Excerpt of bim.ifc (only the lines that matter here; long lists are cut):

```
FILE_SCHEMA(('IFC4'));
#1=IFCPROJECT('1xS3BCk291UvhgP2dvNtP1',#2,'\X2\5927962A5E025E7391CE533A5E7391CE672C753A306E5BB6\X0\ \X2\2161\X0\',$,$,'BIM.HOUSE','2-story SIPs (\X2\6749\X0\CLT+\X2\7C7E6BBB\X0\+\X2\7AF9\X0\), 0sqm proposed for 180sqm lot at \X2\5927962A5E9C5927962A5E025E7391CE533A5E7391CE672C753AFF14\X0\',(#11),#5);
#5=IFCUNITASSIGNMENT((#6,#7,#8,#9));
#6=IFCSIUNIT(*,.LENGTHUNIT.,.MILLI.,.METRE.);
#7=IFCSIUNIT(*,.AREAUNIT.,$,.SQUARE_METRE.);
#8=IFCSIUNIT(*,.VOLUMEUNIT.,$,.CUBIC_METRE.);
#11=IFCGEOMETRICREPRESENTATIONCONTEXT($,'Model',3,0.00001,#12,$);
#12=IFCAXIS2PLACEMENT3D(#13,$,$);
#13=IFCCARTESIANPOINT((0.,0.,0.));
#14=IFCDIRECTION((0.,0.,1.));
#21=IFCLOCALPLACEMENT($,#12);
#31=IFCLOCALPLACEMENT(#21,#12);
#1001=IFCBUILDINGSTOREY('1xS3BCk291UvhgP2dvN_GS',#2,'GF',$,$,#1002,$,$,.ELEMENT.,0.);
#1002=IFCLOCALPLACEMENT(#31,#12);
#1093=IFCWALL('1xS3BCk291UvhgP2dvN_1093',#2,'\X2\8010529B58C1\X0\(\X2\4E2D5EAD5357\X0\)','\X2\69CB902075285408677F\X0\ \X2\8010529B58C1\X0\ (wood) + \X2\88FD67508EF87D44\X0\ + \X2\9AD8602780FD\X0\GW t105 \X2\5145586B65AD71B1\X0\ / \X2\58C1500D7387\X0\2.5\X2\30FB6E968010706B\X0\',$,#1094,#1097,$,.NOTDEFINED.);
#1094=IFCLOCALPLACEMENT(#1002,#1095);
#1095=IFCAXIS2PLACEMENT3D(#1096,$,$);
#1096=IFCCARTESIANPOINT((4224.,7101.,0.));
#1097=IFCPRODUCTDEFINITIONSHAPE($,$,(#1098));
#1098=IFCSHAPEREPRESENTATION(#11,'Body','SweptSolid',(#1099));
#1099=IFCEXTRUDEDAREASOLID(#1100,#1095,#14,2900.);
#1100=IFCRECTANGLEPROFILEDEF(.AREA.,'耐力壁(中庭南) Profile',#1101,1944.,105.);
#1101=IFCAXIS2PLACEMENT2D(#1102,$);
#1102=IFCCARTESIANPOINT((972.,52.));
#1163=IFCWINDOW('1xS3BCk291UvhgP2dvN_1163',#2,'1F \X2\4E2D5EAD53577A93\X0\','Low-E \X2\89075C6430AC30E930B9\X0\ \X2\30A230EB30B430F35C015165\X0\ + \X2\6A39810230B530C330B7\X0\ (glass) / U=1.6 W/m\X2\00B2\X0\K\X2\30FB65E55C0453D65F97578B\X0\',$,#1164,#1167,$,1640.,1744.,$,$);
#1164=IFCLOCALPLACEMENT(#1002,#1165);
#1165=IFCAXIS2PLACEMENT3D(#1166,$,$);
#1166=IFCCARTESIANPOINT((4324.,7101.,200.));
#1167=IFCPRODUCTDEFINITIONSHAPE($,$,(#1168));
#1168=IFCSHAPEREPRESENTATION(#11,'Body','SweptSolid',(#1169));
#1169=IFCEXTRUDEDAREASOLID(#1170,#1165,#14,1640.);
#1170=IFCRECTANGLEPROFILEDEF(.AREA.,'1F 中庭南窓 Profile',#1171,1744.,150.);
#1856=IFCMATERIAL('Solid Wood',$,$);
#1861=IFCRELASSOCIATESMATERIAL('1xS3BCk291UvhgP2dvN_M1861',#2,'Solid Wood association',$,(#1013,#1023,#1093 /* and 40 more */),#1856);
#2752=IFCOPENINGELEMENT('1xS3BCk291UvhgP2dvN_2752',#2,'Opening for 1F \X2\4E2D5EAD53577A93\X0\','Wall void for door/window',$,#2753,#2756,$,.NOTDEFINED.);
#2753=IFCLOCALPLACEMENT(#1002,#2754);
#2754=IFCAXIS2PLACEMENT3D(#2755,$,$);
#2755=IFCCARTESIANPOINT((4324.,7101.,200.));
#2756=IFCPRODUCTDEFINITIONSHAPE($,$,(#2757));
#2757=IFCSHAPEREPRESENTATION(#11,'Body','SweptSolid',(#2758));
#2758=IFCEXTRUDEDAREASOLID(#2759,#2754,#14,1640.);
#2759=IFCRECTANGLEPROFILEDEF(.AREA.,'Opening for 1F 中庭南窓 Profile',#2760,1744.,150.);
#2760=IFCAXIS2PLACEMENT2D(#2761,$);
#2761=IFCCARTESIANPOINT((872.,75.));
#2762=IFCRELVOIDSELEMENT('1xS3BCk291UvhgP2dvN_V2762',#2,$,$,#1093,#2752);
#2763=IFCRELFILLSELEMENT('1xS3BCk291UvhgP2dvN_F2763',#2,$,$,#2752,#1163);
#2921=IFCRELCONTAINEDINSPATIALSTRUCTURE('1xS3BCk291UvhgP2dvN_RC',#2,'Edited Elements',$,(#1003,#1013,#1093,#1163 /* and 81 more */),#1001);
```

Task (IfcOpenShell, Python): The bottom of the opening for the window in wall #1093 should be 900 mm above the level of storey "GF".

```python
import numpy as np
import ifcopenshell
import ifcopenshell.api.geometry
import ifcopenshell.geom
import ifcopenshell.util.element
import ifcopenshell.util.placement
import ifcopenshell.util.shape
import ifcopenshell.util.unit

model = ifcopenshell.open("bim.ifc")
unit_scale = ifcopenshell.util.unit.calculate_unit_scale(model)

window = model.by_guid("1xS3BCk291UvhgP2dvN_1163")
opening = window.FillsVoids[0].RelatingOpeningElement
storey = ifcopenshell.util.element.get_container(window, ifc_class="IfcBuildingStorey")
level = ifcopenshell.util.placement.get_local_placement(storey.ObjectPlacement)[2, 3]

# The opening's origin need not be at the sill, so measure its lowest point.
shape = ifcopenshell.geom.create_shape(ifcopenshell.geom.settings(), opening)
bottom = ifcopenshell.util.shape.get_shape_bottom_elevation(shape, shape.geometry) / unit_scale
dz = level + 0.9 / unit_scale - bottom

shift = np.array([0.0, 0.0, dz])
# The window is not placed relative to its opening, so move both.
for product in (opening, window):
    matrix = ifcopenshell.util.placement.get_local_placement(product.ObjectPlacement)
    matrix[:3, 3] += shift
    ifcopenshell.api.geometry.edit_object_placement(model, product=product, matrix=matrix, is_si=False)

print(f"moved by {dz * unit_scale:+.3f} m")

model.write("bim_rev.ifc")
```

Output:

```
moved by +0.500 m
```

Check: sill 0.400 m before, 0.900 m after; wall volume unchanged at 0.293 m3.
